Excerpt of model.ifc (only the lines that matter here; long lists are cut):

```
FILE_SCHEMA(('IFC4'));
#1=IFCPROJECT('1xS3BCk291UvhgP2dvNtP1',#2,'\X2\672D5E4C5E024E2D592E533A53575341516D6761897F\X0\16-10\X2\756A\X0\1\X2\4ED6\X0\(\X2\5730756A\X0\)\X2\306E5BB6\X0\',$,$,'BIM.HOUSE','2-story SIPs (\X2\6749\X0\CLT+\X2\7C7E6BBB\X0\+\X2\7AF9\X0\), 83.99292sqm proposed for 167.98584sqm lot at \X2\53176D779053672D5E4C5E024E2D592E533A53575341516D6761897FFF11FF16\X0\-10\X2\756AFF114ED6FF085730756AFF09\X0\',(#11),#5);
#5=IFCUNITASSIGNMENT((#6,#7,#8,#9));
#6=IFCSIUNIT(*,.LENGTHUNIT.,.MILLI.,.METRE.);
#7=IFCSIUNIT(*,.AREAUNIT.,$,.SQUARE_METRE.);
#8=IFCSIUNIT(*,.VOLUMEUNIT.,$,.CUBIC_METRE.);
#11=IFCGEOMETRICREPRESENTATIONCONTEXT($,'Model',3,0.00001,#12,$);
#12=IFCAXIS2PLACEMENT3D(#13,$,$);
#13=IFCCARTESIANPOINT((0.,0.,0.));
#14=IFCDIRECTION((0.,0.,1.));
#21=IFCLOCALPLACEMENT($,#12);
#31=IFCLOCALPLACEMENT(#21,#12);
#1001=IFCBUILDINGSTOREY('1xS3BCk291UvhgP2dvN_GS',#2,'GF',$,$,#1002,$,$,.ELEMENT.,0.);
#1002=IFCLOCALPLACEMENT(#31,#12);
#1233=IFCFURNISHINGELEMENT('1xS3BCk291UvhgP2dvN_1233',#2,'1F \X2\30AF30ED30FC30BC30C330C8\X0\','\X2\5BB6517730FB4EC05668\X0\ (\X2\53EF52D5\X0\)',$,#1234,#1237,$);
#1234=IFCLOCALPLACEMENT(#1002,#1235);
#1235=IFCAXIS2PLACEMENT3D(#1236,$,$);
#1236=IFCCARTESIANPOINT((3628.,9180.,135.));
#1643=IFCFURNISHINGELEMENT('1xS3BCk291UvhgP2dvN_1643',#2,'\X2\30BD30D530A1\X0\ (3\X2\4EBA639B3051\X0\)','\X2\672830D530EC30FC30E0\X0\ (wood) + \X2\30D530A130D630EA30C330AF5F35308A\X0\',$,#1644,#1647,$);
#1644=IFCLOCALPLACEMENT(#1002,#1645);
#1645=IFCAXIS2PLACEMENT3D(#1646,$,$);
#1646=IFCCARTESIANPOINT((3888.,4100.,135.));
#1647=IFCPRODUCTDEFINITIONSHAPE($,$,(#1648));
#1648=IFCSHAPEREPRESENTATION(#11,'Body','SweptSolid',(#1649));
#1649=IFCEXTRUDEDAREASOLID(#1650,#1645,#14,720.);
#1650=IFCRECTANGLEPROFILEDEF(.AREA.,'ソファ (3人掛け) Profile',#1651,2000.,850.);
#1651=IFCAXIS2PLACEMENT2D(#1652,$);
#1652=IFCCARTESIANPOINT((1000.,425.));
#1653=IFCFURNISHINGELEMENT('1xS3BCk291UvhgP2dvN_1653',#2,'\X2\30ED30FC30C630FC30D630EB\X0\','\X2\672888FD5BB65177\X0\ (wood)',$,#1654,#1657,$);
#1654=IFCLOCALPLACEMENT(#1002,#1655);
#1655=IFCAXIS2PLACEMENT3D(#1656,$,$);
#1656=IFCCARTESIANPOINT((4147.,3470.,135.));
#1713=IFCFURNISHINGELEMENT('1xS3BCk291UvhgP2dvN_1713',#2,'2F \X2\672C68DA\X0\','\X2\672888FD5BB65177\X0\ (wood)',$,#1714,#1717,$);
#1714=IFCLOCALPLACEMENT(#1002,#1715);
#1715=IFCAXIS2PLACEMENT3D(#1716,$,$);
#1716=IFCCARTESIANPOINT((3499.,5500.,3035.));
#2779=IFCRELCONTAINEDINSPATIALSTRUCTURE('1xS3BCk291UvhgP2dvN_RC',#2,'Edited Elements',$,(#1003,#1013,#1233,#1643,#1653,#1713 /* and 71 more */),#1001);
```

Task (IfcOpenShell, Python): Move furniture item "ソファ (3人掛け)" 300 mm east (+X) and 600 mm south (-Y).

```python
import ifcopenshell
import ifcopenshell.api.geometry
import ifcopenshell.util.placement
import ifcopenshell.util.unit

model = ifcopenshell.open("model.ifc")
unit_scale = ifcopenshell.util.unit.calculate_unit_scale(model)

item = model.by_guid("1xS3BCk291UvhgP2dvN_1643")
matrix = ifcopenshell.util.placement.get_local_placement(item.ObjectPlacement)
matrix[0, 3] += 0.3 / unit_scale
matrix[1, 3] -= 0.6 / unit_scale
ifcopenshell.api.geometry.edit_object_placement(model, product=item, matrix=matrix, is_si=False)

print(ifcopenshell.util.placement.get_local_placement(item.ObjectPlacement).round(3) + 0.0)

model.write("model_edited.ifc")
```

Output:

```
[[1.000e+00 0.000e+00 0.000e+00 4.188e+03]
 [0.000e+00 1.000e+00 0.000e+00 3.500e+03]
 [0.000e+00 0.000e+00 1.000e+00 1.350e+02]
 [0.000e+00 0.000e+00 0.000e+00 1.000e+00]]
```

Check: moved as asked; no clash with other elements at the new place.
